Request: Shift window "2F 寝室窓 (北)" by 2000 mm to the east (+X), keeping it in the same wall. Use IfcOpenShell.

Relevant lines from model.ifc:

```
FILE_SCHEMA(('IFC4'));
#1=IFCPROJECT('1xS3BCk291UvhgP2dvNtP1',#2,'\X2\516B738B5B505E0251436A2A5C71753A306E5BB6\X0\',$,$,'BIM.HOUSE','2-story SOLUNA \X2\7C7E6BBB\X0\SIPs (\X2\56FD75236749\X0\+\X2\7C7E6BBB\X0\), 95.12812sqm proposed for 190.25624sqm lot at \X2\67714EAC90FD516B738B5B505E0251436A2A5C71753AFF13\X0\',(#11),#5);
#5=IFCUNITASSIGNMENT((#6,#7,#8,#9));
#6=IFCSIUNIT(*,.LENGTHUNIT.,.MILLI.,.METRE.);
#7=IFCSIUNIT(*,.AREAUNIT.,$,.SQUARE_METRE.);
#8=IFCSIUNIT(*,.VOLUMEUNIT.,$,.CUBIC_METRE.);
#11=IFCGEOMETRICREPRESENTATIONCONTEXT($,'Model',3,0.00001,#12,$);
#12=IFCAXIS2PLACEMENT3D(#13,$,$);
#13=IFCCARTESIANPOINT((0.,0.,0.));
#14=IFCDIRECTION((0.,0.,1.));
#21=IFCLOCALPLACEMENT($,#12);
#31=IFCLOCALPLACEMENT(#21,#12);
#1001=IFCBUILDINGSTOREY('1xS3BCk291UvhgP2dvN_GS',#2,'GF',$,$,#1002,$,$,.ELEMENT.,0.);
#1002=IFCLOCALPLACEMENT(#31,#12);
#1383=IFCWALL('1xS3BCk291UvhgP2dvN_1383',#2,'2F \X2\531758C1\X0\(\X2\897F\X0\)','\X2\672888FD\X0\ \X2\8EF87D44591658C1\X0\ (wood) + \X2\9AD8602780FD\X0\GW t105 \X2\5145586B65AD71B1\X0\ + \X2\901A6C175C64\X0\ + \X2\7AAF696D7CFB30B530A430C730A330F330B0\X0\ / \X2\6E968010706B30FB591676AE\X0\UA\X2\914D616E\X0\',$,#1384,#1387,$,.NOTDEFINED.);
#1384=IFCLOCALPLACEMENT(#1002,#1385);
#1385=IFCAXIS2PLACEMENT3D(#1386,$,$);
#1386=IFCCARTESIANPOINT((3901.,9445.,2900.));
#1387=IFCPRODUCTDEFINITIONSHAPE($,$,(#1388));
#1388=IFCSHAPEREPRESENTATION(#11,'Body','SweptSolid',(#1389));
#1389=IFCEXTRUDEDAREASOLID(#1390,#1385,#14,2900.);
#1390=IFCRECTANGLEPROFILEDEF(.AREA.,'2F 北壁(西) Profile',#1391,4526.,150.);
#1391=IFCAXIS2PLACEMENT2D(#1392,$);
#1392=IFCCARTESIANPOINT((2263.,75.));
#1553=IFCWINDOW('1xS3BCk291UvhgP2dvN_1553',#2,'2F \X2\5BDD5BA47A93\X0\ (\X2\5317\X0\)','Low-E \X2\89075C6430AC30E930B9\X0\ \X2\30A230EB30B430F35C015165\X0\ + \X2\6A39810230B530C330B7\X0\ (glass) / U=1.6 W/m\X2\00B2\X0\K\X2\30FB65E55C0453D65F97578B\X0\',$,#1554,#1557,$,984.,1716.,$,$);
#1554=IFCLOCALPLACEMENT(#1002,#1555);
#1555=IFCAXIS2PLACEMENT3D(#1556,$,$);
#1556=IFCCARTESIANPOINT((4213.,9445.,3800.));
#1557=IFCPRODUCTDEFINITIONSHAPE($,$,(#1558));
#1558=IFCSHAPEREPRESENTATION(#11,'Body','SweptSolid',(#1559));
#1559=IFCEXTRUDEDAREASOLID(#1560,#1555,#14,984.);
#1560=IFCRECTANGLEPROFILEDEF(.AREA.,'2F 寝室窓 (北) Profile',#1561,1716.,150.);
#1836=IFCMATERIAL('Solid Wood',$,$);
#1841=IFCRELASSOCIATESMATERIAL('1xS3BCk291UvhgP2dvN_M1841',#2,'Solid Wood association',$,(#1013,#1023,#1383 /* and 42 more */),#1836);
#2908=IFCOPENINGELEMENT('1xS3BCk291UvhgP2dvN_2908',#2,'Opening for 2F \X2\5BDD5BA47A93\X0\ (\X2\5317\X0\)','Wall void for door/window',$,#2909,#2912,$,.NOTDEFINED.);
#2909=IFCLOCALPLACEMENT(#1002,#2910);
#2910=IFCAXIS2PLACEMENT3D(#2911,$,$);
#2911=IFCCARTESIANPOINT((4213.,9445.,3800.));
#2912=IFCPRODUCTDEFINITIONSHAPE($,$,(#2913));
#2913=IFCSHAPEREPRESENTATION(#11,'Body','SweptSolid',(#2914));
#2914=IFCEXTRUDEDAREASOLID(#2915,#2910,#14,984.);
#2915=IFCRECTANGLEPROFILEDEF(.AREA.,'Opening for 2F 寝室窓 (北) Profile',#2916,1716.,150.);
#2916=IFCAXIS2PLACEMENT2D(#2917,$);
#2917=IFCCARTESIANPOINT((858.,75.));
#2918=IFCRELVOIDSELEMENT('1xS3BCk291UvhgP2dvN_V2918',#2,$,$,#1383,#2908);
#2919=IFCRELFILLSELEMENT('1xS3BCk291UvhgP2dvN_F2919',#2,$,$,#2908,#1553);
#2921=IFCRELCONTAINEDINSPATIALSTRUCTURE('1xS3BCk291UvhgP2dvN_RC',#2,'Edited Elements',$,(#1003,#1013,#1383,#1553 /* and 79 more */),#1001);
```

```python
import ifcopenshell
import ifcopenshell.api.geometry
import ifcopenshell.util.placement

model = ifcopenshell.open("model.ifc")

window = model.by_guid("1xS3BCk291UvhgP2dvN_1553")
opening = window.FillsVoids[0].RelatingOpeningElement
wall = opening.VoidsElements[0].RelatingBuildingElement

wall_matrix = ifcopenshell.util.placement.get_local_placement(wall.ObjectPlacement)
shift = wall_matrix[:3, 0] * 2000.0
before = ifcopenshell.util.placement.get_local_placement(window.ObjectPlacement)[:3, 3].copy()

# The window is not placed relative to its opening, so move both.
for product in (opening, window):
    matrix = ifcopenshell.util.placement.get_local_placement(product.ObjectPlacement)
    matrix[:3, 3] += shift
    ifcopenshell.api.geometry.edit_object_placement(model, product=product, matrix=matrix, is_si=False)

after = ifcopenshell.util.placement.get_local_placement(window.ObjectPlacement)[:3, 3]
print("window moved by", (after - before).round(3) + 0.0)

model.write("model_updated.ifc")
```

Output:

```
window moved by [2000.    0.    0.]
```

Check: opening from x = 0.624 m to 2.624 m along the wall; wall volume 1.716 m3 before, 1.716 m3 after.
